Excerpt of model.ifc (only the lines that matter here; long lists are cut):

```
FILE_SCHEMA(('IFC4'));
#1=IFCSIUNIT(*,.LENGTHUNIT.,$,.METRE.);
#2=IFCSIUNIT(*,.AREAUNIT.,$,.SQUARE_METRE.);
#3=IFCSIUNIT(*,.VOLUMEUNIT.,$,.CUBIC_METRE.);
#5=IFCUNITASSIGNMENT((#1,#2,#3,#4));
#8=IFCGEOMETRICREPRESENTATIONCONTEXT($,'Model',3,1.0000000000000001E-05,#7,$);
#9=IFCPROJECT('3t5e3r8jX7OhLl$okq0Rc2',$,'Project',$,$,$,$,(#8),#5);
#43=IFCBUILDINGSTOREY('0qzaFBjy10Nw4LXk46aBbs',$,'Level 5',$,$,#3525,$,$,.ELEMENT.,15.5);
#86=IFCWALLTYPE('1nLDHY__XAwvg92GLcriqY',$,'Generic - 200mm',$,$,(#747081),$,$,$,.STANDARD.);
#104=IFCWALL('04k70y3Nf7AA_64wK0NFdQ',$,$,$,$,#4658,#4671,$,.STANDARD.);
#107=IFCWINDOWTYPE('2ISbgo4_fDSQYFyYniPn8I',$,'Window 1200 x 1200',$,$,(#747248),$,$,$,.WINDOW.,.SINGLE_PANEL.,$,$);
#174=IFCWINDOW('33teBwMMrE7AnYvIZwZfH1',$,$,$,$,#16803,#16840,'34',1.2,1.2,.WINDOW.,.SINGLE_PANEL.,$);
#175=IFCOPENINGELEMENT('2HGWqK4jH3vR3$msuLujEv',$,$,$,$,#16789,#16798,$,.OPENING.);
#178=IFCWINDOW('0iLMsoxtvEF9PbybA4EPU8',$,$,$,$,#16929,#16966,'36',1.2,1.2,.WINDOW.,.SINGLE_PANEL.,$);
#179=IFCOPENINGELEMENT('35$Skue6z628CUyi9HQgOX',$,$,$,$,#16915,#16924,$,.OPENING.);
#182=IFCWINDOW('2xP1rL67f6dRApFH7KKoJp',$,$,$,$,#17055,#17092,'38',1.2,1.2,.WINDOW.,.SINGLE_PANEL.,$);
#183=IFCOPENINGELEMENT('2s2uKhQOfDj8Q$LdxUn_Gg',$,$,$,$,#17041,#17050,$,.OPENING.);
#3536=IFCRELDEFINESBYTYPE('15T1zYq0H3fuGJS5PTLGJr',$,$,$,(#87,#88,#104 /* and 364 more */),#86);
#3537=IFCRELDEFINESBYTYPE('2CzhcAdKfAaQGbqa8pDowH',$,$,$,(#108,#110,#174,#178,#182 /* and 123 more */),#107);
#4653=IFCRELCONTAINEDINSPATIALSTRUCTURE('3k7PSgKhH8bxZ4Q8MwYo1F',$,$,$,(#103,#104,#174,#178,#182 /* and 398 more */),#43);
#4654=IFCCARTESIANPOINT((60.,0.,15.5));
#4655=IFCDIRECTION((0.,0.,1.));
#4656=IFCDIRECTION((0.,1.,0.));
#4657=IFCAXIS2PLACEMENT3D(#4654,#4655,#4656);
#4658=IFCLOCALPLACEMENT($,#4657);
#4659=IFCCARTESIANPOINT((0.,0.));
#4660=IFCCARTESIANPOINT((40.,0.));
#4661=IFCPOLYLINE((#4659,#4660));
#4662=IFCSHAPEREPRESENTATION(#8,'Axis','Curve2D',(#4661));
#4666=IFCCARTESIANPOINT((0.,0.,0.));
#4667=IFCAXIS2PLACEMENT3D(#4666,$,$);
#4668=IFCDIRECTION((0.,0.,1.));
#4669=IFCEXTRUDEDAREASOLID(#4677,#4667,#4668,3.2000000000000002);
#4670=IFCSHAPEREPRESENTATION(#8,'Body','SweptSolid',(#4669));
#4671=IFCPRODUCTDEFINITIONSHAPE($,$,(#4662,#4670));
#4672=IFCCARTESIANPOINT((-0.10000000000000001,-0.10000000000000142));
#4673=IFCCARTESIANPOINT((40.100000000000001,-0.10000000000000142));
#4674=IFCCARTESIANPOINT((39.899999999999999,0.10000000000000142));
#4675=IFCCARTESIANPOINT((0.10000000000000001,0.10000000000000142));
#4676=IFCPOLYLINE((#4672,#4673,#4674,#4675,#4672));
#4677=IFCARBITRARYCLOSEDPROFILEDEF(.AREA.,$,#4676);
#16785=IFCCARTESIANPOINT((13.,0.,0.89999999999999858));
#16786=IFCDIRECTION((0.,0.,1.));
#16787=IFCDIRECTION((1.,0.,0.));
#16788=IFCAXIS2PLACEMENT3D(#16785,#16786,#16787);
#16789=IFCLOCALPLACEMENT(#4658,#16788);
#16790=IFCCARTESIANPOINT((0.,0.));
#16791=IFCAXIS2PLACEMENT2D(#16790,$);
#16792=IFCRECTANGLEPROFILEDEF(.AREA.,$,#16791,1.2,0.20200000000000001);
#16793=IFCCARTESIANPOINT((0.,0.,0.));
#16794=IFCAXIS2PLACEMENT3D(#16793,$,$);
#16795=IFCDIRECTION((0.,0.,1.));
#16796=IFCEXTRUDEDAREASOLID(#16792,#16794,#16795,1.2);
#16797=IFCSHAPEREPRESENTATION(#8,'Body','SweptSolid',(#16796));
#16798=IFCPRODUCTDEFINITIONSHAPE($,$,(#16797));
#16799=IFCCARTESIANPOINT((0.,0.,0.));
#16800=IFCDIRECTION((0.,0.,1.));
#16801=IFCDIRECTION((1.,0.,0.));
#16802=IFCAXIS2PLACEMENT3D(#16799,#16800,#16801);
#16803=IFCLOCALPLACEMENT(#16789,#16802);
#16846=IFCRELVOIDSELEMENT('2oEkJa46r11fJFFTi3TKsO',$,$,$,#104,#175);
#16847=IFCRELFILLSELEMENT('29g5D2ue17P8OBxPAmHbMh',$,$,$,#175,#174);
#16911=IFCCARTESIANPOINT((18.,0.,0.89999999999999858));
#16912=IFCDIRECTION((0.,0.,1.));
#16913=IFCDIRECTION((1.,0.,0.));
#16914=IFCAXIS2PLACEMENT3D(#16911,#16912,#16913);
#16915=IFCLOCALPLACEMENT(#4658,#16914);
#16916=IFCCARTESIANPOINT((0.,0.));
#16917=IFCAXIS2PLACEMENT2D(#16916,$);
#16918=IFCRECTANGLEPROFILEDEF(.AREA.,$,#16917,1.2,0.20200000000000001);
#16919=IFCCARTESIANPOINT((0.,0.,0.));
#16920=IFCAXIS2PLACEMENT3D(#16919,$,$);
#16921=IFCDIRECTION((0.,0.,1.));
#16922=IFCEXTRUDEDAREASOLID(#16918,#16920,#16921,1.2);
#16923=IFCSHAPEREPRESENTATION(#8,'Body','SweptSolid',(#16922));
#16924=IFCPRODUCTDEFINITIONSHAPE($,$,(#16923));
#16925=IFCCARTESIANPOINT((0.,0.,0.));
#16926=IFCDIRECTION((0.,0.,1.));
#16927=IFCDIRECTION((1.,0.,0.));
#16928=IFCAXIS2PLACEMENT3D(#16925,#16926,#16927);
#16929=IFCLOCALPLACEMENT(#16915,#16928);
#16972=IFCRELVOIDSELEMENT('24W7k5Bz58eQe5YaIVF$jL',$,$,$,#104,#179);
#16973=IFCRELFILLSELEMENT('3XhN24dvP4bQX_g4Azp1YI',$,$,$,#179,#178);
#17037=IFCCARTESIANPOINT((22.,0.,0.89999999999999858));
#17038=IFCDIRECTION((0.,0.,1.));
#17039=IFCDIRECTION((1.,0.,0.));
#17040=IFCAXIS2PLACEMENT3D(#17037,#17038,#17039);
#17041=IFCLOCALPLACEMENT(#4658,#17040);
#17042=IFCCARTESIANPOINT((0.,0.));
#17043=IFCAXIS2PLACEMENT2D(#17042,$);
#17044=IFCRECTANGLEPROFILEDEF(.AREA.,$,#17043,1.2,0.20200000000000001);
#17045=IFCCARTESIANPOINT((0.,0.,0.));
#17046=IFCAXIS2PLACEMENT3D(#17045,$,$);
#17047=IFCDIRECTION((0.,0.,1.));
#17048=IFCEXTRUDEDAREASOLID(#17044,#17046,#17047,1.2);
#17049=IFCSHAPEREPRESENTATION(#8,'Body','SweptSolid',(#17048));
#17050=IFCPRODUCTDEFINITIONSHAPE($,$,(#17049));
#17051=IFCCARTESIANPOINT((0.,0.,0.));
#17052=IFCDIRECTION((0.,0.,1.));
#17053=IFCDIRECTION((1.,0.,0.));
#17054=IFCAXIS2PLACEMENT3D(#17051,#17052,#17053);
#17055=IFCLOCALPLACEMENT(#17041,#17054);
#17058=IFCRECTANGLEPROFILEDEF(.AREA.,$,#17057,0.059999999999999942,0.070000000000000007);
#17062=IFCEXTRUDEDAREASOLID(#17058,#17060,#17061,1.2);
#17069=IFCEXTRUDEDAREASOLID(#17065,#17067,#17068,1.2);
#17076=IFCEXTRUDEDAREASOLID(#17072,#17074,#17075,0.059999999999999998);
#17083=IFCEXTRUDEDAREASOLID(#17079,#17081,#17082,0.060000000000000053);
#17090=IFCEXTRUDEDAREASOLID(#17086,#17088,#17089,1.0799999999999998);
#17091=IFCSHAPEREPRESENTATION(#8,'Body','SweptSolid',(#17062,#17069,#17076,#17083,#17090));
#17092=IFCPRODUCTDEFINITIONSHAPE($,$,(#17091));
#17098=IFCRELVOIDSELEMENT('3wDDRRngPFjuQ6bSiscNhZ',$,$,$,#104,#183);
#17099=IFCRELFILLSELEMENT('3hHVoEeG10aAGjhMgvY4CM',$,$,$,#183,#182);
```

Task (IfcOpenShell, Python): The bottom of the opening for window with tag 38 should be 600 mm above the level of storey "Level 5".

```python
import numpy as np
import ifcopenshell
import ifcopenshell.api.geometry
import ifcopenshell.geom
import ifcopenshell.util.element
import ifcopenshell.util.placement
import ifcopenshell.util.shape
import ifcopenshell.util.unit

model = ifcopenshell.open("model.ifc")
unit_scale = ifcopenshell.util.unit.calculate_unit_scale(model)

window = model.by_guid("2xP1rL67f6dRApFH7KKoJp")
opening = window.FillsVoids[0].RelatingOpeningElement
storey = ifcopenshell.util.element.get_container(window, ifc_class="IfcBuildingStorey")
level = ifcopenshell.util.placement.get_local_placement(storey.ObjectPlacement)[2, 3]

# The opening's origin need not be at the sill, so measure its lowest point.
shape = ifcopenshell.geom.create_shape(ifcopenshell.geom.settings(), opening)
bottom = ifcopenshell.util.shape.get_shape_bottom_elevation(shape, shape.geometry) / unit_scale
dz = level + 0.6 / unit_scale - bottom

shift = np.array([0.0, 0.0, dz])
# The window is placed relative to its opening, so it follows when the opening moves.
matrix = ifcopenshell.util.placement.get_local_placement(opening.ObjectPlacement)
matrix[:3, 3] += shift
ifcopenshell.api.geometry.edit_object_placement(
    model, product=opening, matrix=matrix, is_si=False, should_transform_children=True
)

print(f"moved by {dz * unit_scale:+.3f} m")

model.write("model_edited.ifc")
```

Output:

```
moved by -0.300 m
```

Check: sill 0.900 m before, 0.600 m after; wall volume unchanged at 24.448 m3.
